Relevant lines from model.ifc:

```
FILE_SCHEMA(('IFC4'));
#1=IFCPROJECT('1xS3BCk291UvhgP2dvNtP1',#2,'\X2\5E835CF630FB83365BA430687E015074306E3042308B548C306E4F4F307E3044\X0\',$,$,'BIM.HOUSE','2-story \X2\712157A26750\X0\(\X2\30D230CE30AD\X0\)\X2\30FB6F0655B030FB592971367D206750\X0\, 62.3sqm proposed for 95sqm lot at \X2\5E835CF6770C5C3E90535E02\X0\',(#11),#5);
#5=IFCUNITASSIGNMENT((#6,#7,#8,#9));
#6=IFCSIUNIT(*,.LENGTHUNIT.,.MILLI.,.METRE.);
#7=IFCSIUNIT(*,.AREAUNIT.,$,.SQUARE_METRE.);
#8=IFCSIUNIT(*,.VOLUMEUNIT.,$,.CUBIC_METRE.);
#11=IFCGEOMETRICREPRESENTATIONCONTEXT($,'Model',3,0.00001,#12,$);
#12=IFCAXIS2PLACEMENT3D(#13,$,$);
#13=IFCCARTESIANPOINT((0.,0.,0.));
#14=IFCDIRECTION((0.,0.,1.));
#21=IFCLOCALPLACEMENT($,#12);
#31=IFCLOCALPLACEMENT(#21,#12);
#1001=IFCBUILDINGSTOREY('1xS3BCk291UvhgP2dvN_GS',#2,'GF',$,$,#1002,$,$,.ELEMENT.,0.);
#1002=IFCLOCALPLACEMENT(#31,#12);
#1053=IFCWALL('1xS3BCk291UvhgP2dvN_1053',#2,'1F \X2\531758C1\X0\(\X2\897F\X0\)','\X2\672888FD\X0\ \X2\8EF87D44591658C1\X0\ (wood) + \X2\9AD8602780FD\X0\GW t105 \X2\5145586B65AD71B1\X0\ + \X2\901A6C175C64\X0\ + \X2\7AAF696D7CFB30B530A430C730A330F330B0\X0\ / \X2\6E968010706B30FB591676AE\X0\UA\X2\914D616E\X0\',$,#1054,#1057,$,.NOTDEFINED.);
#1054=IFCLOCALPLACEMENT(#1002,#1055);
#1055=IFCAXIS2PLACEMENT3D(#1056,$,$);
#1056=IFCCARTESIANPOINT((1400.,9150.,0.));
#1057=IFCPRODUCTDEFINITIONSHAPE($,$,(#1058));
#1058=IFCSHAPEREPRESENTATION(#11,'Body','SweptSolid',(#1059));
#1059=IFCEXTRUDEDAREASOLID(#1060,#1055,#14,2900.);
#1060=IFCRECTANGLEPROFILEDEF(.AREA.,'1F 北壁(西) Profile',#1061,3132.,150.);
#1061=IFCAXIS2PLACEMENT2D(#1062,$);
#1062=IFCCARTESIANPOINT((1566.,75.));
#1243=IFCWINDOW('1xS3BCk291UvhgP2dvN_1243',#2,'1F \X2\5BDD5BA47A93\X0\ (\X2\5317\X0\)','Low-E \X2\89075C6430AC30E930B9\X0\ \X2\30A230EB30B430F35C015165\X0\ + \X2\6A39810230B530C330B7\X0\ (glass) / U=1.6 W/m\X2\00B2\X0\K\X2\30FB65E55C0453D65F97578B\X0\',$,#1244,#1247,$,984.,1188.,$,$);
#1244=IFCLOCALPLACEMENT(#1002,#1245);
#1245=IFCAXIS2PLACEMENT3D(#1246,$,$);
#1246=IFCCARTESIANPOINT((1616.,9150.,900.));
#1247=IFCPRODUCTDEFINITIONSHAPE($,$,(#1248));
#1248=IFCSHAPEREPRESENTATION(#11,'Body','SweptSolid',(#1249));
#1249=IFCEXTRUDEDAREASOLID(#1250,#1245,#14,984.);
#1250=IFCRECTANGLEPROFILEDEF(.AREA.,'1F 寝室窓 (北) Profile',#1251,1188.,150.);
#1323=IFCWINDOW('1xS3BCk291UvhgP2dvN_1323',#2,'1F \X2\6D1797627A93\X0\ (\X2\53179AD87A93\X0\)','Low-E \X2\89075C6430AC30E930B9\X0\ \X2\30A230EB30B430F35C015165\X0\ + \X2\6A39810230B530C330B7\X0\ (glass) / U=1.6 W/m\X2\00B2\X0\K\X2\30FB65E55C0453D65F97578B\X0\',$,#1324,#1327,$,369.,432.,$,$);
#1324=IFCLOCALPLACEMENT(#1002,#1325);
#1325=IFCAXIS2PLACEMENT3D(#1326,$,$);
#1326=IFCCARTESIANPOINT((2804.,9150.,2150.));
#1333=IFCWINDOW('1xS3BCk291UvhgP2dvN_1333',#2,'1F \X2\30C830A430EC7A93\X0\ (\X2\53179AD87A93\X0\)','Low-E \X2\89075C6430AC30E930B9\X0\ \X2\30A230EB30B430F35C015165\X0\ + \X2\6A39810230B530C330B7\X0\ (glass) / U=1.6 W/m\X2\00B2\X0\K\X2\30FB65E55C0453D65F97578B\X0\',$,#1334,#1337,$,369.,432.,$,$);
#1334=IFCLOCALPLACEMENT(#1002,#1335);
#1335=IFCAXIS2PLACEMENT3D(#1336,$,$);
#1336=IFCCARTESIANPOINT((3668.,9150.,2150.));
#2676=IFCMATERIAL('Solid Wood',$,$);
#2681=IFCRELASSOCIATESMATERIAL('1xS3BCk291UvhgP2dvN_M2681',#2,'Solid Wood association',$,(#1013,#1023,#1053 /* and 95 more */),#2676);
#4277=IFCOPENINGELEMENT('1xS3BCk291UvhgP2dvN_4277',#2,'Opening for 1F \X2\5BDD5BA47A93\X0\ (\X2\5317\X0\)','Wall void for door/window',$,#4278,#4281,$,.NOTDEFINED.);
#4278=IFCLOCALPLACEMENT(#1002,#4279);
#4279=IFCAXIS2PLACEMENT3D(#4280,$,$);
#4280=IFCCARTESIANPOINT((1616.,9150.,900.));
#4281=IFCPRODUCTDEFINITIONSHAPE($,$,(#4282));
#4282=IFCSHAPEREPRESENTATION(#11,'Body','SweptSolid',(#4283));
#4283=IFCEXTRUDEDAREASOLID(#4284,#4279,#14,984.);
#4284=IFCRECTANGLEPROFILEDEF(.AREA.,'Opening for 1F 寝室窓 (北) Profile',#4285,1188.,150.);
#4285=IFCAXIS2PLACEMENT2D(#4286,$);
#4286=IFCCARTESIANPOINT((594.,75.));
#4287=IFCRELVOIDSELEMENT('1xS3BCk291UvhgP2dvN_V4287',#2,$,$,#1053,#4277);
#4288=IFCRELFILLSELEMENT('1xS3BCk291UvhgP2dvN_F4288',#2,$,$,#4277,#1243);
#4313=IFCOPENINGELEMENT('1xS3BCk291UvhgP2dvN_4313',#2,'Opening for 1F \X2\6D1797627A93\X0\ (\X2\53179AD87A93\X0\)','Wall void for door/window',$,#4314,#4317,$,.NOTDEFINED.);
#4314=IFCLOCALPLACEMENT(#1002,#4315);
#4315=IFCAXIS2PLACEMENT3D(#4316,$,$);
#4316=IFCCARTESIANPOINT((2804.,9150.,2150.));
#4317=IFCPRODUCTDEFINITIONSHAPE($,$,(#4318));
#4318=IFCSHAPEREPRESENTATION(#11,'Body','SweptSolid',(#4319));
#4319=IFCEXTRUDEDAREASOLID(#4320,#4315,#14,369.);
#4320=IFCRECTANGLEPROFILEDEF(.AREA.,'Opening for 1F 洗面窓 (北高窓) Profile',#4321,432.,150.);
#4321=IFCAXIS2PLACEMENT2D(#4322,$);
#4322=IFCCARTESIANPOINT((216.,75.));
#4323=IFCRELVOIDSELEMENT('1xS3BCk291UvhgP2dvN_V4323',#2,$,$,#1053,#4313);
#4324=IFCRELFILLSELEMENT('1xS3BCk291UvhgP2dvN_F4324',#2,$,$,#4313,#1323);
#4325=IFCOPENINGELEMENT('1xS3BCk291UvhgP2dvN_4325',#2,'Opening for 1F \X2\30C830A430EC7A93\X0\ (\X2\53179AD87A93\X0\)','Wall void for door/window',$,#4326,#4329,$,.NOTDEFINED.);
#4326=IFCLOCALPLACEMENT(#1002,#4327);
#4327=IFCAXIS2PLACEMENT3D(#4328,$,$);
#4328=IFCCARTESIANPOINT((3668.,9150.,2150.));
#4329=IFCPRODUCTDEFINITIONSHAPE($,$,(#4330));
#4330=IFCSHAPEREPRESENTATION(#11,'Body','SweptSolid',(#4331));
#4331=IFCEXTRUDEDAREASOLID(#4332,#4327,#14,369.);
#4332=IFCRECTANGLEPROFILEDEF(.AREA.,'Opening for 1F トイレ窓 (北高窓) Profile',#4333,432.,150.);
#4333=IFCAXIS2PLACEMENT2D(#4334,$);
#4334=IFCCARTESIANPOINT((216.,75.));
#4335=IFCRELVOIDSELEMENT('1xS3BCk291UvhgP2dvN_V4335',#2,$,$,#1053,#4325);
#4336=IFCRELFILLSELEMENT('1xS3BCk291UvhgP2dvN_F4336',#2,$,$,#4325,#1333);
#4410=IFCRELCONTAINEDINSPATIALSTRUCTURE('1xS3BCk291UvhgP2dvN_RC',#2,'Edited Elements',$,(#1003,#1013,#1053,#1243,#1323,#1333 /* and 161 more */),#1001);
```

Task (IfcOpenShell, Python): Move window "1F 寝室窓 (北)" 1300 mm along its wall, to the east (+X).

```python
import ifcopenshell
import ifcopenshell.api.geometry
import ifcopenshell.util.placement
import ifcopenshell.util.unit

model = ifcopenshell.open("model.ifc")
unit_scale = ifcopenshell.util.unit.calculate_unit_scale(model)

window = model.by_id(1243)
opening = window.FillsVoids[0].RelatingOpeningElement
wall = opening.VoidsElements[0].RelatingBuildingElement

wall_matrix = ifcopenshell.util.placement.get_local_placement(wall.ObjectPlacement)
shift = wall_matrix[:3, 0] * 1.3 / unit_scale
before = ifcopenshell.util.placement.get_local_placement(window.ObjectPlacement)[:3, 3].copy()

# The window is not placed relative to its opening, so move both.
for product in (opening, window):
    matrix = ifcopenshell.util.placement.get_local_placement(product.ObjectPlacement)
    matrix[:3, 3] += shift
    ifcopenshell.api.geometry.edit_object_placement(model, product=product, matrix=matrix, is_si=False)

after = ifcopenshell.util.placement.get_local_placement(window.ObjectPlacement)[:3, 3]
print("window moved by", (after - before).round(3) + 0.0)

model.write("model_rev.ifc")
```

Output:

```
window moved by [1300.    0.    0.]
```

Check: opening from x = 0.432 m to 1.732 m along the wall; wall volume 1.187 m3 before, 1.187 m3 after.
